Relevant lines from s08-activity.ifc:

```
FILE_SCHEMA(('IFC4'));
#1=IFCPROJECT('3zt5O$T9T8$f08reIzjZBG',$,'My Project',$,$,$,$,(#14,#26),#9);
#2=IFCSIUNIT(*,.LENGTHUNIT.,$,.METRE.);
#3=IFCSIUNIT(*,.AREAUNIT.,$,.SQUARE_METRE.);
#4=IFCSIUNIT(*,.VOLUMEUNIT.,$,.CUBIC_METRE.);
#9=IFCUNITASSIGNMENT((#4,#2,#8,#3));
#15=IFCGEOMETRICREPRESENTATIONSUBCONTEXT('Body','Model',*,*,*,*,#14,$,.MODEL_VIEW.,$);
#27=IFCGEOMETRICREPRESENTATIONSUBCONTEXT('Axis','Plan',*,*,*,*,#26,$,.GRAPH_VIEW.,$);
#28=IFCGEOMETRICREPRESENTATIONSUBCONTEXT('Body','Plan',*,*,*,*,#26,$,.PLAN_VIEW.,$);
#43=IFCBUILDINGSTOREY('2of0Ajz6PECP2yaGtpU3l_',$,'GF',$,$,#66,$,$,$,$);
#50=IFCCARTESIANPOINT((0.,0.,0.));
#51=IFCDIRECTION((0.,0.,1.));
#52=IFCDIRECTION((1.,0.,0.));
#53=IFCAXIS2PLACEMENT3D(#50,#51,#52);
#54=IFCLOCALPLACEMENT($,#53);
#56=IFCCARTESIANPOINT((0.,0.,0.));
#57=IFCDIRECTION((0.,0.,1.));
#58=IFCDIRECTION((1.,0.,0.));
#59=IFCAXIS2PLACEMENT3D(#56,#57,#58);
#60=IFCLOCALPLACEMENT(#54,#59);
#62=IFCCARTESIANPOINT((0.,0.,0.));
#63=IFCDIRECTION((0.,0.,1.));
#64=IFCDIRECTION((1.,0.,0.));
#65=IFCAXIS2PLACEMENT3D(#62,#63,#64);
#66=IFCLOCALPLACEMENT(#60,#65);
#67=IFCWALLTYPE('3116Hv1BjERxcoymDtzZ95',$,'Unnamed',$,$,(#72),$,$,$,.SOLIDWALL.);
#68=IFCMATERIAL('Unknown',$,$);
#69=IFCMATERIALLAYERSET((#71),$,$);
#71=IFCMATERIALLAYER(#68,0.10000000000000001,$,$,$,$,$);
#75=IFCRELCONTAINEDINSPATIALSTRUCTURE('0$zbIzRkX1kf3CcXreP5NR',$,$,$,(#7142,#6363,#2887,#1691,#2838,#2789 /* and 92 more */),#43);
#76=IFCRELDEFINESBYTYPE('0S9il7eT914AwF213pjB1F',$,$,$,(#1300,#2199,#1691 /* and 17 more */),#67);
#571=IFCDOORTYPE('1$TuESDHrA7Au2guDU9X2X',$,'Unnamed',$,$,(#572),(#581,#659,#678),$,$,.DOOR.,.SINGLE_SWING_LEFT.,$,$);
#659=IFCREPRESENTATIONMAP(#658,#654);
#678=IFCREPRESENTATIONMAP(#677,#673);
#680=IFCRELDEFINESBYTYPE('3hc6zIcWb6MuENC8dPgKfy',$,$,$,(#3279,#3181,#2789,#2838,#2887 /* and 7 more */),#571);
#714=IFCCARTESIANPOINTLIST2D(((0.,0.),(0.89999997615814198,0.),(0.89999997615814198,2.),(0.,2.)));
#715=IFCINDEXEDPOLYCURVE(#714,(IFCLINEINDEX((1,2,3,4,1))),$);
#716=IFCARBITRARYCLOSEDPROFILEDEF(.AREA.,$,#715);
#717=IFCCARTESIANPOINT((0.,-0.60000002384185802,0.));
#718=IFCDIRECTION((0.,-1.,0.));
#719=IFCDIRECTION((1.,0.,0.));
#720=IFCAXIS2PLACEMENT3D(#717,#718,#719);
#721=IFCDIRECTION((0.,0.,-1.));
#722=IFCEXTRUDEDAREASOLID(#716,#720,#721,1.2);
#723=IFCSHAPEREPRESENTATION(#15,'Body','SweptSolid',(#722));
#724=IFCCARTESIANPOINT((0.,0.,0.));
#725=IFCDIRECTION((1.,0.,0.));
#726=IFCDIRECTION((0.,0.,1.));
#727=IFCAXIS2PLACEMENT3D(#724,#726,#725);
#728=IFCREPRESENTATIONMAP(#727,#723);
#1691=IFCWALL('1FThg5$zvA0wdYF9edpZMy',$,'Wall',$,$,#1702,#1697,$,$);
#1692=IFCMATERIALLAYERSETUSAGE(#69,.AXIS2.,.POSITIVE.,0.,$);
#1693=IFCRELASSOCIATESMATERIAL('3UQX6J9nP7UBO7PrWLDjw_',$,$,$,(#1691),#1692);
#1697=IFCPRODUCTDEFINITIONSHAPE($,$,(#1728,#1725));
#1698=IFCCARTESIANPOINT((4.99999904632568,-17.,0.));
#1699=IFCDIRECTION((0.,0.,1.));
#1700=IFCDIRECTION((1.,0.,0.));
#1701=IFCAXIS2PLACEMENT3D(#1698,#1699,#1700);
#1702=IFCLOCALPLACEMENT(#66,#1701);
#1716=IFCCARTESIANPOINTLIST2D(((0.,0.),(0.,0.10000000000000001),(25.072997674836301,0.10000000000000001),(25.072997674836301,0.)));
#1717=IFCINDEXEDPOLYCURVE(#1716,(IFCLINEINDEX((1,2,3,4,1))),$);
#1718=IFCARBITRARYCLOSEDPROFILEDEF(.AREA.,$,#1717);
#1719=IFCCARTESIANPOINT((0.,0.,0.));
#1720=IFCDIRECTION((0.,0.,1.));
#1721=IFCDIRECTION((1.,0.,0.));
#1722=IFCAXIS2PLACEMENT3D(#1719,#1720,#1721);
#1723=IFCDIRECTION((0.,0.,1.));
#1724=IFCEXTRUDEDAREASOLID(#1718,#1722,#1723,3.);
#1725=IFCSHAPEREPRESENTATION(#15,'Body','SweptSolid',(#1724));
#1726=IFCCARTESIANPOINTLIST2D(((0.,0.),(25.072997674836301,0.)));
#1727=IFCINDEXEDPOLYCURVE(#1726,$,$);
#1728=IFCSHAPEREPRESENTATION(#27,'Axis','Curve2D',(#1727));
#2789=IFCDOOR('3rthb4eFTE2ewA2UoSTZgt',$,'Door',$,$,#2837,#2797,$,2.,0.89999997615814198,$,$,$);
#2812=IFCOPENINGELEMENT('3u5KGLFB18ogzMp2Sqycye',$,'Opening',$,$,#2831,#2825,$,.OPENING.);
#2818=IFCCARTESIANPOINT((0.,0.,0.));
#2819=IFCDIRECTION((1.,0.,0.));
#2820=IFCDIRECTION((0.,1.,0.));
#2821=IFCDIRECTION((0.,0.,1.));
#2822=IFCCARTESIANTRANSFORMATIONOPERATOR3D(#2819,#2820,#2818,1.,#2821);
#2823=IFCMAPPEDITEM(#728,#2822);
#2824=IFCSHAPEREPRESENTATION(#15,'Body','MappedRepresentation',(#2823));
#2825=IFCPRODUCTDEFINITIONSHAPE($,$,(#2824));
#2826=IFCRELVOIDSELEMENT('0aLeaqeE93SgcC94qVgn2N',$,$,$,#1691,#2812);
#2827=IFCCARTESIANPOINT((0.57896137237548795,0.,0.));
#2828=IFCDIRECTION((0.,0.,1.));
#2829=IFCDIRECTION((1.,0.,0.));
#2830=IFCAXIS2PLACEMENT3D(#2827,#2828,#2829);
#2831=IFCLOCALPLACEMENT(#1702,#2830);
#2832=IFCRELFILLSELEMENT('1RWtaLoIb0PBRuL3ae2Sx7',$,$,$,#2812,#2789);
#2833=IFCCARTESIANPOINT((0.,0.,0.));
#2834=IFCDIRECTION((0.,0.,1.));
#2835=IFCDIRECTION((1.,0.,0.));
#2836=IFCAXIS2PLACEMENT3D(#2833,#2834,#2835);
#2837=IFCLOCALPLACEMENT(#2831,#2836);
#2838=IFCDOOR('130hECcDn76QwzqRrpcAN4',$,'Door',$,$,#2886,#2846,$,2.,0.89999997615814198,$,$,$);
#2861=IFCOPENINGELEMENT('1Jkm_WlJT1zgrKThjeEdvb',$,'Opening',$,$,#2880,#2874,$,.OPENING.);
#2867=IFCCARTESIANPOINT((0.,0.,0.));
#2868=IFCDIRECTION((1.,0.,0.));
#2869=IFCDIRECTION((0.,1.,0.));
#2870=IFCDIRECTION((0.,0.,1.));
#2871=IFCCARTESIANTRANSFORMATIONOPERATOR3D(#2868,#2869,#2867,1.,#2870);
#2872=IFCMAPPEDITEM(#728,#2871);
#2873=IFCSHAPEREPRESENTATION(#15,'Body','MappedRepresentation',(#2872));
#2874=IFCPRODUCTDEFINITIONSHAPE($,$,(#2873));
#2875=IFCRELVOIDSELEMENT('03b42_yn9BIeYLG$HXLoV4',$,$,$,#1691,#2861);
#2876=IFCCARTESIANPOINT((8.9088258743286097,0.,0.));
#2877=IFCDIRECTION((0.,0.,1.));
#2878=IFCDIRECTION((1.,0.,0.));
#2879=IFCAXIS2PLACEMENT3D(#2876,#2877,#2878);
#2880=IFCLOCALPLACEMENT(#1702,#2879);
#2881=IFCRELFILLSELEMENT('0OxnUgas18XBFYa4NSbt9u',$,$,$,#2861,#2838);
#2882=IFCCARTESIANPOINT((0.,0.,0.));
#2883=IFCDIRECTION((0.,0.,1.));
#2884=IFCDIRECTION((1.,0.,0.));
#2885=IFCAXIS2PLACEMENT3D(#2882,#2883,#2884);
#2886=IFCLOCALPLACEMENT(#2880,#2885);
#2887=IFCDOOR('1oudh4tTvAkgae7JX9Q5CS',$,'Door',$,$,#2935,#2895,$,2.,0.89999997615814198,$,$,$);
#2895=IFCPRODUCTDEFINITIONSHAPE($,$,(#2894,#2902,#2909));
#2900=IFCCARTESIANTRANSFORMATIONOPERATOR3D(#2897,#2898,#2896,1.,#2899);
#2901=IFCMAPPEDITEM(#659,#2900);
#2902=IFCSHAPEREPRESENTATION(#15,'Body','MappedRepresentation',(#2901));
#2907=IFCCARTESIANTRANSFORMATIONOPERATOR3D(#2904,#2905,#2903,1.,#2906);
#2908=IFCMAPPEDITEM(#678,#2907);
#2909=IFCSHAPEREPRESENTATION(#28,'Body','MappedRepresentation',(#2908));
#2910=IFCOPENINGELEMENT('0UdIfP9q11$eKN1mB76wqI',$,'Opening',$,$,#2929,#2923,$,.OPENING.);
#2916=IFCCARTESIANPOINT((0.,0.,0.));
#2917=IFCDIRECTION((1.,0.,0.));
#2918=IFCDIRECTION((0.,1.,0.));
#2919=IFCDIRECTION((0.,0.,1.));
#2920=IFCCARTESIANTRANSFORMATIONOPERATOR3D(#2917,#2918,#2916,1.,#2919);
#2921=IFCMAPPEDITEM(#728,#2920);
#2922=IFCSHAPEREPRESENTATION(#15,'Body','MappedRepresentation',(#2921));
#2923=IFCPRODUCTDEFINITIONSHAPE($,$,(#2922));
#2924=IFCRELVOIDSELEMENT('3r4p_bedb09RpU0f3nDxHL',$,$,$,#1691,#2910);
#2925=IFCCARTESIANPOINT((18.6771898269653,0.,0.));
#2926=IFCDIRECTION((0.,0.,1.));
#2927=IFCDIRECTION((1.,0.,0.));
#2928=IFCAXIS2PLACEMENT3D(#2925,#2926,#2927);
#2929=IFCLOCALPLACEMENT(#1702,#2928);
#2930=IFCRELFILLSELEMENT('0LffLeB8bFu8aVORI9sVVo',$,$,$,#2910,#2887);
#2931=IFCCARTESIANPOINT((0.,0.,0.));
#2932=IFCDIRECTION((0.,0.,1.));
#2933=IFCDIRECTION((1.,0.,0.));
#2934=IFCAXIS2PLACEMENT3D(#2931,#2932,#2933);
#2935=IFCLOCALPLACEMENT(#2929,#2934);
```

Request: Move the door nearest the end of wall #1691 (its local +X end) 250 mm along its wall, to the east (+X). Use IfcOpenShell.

```python
import ifcopenshell
import ifcopenshell.api.geometry
import ifcopenshell.util.placement
import ifcopenshell.util.unit

model = ifcopenshell.open("s08-activity.ifc")
unit_scale = ifcopenshell.util.unit.calculate_unit_scale(model)

door = model.by_guid("1oudh4tTvAkgae7JX9Q5CS")
opening = door.FillsVoids[0].RelatingOpeningElement
wall = opening.VoidsElements[0].RelatingBuildingElement

wall_matrix = ifcopenshell.util.placement.get_local_placement(wall.ObjectPlacement)
shift = wall_matrix[:3, 0] * 0.25 / unit_scale
before = ifcopenshell.util.placement.get_local_placement(door.ObjectPlacement)[:3, 3].copy()

# The door is placed relative to its opening, so it follows when the opening moves.
matrix = ifcopenshell.util.placement.get_local_placement(opening.ObjectPlacement)
matrix[:3, 3] += shift
ifcopenshell.api.geometry.edit_object_placement(
    model, product=opening, matrix=matrix, is_si=False, should_transform_children=True
)

after = ifcopenshell.util.placement.get_local_placement(door.ObjectPlacement)[:3, 3]
print("door moved by", (after - before).round(3) + 0.0)

model.write("s08-activity_edited.ifc")
```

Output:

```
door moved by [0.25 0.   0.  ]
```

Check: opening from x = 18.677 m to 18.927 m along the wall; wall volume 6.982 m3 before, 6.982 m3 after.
